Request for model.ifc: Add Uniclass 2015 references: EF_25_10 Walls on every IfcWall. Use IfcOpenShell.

First a look at what the model holds.

```python
import ifcopenshell

model = ifcopenshell.open("model.ifc")
print(model.schema)
print("classifications:", [c.Name for c in model.by_type("IfcClassification")])
for ifc_class in ("IfcDoor", "IfcRoof", "IfcStair", "IfcWall", "IfcWindow"):
    print(ifc_class, len(model.by_type(ifc_class)))
```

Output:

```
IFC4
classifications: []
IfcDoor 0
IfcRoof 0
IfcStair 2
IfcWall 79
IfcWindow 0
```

```python
import ifcopenshell
import ifcopenshell.api.classification

model = ifcopenshell.open("model.ifc")

system = ifcopenshell.api.classification.add_classification(model, classification="Uniclass 2015")

codes = {
    "IfcWall": ("EF_25_10", "Walls"),
}
for ifc_class, (code, name) in codes.items():
    products = model.by_type(ifc_class)
    ifcopenshell.api.classification.add_reference(
        model, products=products, classification=system, identification=code, name=name
    )
    print(code, len(products))

model.write("model_edited.ifc")
```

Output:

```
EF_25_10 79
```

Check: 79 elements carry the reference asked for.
